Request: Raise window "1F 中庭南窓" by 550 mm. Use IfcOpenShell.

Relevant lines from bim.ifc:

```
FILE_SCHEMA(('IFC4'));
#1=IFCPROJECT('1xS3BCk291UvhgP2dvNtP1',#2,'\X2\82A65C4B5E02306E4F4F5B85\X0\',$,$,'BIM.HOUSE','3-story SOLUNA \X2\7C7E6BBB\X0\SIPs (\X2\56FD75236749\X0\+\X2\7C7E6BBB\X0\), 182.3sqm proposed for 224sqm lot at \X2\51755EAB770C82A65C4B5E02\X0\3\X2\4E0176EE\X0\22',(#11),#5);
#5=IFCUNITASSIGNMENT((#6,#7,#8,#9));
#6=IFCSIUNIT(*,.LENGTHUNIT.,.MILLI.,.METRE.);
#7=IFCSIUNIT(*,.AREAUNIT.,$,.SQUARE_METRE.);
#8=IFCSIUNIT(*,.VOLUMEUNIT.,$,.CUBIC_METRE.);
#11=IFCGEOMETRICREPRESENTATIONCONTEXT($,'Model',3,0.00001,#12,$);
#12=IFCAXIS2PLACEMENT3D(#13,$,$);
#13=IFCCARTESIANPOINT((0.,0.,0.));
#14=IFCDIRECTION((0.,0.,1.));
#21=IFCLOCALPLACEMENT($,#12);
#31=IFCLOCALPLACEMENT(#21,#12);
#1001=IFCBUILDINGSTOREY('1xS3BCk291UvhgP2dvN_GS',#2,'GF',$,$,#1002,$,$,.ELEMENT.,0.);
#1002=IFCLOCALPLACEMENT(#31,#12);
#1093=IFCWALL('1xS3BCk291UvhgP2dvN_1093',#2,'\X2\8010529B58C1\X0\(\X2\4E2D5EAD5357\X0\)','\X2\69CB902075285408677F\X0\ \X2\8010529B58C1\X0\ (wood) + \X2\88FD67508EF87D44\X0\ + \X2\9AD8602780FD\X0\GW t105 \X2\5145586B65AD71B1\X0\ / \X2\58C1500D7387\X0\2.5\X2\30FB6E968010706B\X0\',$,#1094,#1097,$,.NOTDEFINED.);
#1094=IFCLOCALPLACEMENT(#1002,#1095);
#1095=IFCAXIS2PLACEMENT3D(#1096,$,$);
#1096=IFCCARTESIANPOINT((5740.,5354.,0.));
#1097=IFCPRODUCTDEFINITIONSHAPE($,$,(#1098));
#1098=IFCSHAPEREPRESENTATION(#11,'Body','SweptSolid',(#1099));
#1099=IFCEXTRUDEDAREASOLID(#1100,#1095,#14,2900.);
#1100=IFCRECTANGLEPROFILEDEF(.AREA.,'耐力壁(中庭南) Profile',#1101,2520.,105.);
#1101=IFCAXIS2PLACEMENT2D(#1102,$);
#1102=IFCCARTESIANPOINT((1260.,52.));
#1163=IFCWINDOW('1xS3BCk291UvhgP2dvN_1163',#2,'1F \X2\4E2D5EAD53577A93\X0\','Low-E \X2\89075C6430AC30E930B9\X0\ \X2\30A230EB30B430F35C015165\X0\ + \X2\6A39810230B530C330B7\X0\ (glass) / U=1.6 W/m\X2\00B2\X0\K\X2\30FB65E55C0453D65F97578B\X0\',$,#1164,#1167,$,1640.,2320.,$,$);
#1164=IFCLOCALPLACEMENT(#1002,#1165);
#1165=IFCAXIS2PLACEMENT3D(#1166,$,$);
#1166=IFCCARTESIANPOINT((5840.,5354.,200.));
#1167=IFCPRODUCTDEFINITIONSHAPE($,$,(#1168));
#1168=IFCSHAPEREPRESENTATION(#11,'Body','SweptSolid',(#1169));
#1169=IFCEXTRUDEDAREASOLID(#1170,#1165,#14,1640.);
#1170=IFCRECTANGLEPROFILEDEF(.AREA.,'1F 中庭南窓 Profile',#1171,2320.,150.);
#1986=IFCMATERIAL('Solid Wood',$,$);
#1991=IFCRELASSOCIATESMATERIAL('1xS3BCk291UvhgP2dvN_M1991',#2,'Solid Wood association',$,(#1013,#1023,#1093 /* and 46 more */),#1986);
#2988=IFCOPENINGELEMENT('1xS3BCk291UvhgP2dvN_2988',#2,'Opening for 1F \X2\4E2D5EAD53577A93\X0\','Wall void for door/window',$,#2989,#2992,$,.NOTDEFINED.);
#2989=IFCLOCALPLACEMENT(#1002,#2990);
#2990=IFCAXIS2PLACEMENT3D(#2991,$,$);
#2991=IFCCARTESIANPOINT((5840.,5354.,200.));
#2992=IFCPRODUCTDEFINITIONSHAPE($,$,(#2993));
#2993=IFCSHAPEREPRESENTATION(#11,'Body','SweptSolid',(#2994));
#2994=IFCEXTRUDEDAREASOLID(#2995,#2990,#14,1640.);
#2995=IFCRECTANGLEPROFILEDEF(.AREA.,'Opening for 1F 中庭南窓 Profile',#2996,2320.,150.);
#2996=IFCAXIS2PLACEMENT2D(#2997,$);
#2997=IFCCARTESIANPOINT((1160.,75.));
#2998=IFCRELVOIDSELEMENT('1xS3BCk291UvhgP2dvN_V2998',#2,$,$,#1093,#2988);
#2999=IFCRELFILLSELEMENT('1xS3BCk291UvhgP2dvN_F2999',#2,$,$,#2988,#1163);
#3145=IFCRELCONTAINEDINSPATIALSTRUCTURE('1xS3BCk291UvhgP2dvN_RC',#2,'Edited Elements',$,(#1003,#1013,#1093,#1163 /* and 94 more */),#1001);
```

```python
import numpy as np
import ifcopenshell
import ifcopenshell.api.geometry
import ifcopenshell.util.placement
import ifcopenshell.util.unit

model = ifcopenshell.open("bim.ifc")
unit_scale = ifcopenshell.util.unit.calculate_unit_scale(model)

window = model.by_guid("1xS3BCk291UvhgP2dvN_1163")
opening = window.FillsVoids[0].RelatingOpeningElement
dz = 0.55 / unit_scale

shift = np.array([0.0, 0.0, dz])
# The window is not placed relative to its opening, so move both.
for product in (opening, window):
    matrix = ifcopenshell.util.placement.get_local_placement(product.ObjectPlacement)
    matrix[:3, 3] += shift
    ifcopenshell.api.geometry.edit_object_placement(model, product=product, matrix=matrix, is_si=False)

print(f"moved by {dz * unit_scale:+.3f} m")

model.write("bim_v2.ifc")
```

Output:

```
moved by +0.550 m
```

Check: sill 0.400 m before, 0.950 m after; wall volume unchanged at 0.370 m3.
